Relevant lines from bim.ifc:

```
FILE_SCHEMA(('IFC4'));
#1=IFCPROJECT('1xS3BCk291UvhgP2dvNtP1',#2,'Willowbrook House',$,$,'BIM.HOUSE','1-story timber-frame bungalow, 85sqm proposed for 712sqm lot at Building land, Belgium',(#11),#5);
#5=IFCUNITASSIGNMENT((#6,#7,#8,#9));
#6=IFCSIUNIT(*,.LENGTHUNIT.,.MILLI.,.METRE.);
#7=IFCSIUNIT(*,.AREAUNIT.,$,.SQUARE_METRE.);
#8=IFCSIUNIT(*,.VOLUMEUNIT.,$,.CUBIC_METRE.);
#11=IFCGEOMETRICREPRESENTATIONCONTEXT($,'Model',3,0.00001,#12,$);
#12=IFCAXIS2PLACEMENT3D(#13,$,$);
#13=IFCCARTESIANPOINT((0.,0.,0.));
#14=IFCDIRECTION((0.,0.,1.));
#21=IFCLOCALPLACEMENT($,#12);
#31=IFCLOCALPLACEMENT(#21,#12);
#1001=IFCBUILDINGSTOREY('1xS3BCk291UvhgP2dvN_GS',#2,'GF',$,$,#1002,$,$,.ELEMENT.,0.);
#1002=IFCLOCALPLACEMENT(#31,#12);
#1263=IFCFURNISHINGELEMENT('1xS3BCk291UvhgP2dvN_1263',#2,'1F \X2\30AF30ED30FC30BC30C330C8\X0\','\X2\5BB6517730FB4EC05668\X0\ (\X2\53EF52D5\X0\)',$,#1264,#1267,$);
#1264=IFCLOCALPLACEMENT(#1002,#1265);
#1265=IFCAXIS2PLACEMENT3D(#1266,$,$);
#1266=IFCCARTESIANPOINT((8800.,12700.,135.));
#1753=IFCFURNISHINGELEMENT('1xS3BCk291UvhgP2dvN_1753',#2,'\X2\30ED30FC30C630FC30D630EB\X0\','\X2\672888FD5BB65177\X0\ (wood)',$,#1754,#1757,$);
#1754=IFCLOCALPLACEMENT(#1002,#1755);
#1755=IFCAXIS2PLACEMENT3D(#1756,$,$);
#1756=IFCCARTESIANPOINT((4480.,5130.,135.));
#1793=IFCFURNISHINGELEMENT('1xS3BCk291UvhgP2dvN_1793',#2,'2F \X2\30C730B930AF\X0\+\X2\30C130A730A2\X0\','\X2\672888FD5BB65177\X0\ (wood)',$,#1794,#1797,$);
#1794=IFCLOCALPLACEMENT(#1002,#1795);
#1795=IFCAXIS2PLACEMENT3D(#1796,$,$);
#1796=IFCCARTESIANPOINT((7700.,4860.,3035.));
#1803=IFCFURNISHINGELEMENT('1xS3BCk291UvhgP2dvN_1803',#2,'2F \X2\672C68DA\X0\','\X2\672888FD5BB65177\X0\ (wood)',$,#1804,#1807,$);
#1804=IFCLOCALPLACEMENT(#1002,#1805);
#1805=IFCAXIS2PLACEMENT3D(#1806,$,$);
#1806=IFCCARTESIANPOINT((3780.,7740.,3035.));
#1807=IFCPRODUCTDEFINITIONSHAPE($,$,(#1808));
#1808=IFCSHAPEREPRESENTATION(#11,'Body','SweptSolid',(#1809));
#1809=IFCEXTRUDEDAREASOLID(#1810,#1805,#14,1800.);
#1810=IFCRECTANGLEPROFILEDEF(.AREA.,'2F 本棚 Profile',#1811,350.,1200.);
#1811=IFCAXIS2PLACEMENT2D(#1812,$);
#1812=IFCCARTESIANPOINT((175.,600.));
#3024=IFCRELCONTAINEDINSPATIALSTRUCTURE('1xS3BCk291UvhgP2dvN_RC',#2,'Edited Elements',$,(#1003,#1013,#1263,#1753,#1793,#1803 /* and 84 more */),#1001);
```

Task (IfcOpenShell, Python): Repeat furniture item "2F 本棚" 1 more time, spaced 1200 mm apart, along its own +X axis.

```python
import ifcopenshell
import ifcopenshell.api.geometry
import ifcopenshell.api.root
import ifcopenshell.util.element
import ifcopenshell.util.placement

model = ifcopenshell.open("bim.ifc")


def reuse_history(source, copy):
    """copy_class also copies each property set's owner history, people and application; keep the originals."""
    for rel in copy.IsDefinedBy:
        if rel.is_a("IfcRelDefinesByProperties") and (history := rel.RelatingPropertyDefinition.OwnerHistory):
            rel.RelatingPropertyDefinition.OwnerHistory = source.OwnerHistory
            ifcopenshell.util.element.remove_deep2(model, history)


source = model.by_guid("1xS3BCk291UvhgP2dvN_1803")
base = ifcopenshell.util.placement.get_local_placement(source.ObjectPlacement)
step = base[:3, 0] * 1200.0

for i in range(1, 2):
    copy = ifcopenshell.api.root.copy_class(model, product=source)
    copy.Representation = ifcopenshell.util.element.copy_deep(
        model, source.Representation, exclude=["IfcGeometricRepresentationContext", "IfcRepresentationMap"]
    )
    reuse_history(source, copy)
    matrix = base.copy()
    matrix[:3, 3] += i * step
    print("added at", matrix[:3, 3].round(3) + 0.0)
    ifcopenshell.api.geometry.edit_object_placement(model, product=copy, matrix=matrix, is_si=False)

model.write("bim_rev.ifc")
```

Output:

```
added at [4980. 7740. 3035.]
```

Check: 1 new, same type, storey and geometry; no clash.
